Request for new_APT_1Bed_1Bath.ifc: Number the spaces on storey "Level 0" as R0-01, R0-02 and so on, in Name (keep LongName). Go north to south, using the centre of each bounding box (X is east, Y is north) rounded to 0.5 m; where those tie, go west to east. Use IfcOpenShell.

First a look at what the model holds.

```python
import ifcopenshell
import ifcopenshell.util.element
import ifcopenshell.util.placement

model = ifcopenshell.open("new_APT_1Bed_1Bath.ifc")
print(model.schema)
storey = next(s for s in model.by_type("IfcBuildingStorey") if s.Name == "Level 0")
spaces = [e for e in ifcopenshell.util.element.get_decomposition(storey) if e.is_a("IfcSpace")]
for e in sorted(spaces, key=lambda e: e.id()):
    origin = ifcopenshell.util.placement.get_local_placement(e.ObjectPlacement)[:3, 3]
    print(e.id(), e.Name, e.LongName, origin.round(2) + 0.0, sep=" | ")
```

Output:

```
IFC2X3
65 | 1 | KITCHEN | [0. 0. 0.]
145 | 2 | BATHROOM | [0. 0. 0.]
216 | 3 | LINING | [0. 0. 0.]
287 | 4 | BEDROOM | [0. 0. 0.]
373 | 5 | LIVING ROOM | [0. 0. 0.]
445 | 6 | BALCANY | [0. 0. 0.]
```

```python
import ifcopenshell
import ifcopenshell.geom
import ifcopenshell.util.element
import ifcopenshell.util.shape

model = ifcopenshell.open("new_APT_1Bed_1Bath.ifc")
settings = ifcopenshell.geom.settings()
settings.set("use-world-coords", True)


def centre(element):
    shape = ifcopenshell.geom.create_shape(settings, element)
    return ifcopenshell.util.shape.get_bbox_centroid(shape.geometry)


storey = next(s for s in model.by_type("IfcBuildingStorey") if s.Name == "Level 0")
spaces = [e for e in ifcopenshell.util.element.get_decomposition(storey) if e.is_a("IfcSpace")]

# Insertion points can sit at a corner or the storey origin, so sort by the geometry (in metres).
centres = {e: centre(e) for e in spaces}
spaces.sort(key=lambda e: (-round(centres[e][1] / 0.5), centres[e][0]))

for i, e in enumerate(spaces, start=1):
    number = f"R0-{i:02d}"
    e.Name = number
    print(e.id(), number)

model.write("new_APT_1Bed_1Bath_updated.ifc")
```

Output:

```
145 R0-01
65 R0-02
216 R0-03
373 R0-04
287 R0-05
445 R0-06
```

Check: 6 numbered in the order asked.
